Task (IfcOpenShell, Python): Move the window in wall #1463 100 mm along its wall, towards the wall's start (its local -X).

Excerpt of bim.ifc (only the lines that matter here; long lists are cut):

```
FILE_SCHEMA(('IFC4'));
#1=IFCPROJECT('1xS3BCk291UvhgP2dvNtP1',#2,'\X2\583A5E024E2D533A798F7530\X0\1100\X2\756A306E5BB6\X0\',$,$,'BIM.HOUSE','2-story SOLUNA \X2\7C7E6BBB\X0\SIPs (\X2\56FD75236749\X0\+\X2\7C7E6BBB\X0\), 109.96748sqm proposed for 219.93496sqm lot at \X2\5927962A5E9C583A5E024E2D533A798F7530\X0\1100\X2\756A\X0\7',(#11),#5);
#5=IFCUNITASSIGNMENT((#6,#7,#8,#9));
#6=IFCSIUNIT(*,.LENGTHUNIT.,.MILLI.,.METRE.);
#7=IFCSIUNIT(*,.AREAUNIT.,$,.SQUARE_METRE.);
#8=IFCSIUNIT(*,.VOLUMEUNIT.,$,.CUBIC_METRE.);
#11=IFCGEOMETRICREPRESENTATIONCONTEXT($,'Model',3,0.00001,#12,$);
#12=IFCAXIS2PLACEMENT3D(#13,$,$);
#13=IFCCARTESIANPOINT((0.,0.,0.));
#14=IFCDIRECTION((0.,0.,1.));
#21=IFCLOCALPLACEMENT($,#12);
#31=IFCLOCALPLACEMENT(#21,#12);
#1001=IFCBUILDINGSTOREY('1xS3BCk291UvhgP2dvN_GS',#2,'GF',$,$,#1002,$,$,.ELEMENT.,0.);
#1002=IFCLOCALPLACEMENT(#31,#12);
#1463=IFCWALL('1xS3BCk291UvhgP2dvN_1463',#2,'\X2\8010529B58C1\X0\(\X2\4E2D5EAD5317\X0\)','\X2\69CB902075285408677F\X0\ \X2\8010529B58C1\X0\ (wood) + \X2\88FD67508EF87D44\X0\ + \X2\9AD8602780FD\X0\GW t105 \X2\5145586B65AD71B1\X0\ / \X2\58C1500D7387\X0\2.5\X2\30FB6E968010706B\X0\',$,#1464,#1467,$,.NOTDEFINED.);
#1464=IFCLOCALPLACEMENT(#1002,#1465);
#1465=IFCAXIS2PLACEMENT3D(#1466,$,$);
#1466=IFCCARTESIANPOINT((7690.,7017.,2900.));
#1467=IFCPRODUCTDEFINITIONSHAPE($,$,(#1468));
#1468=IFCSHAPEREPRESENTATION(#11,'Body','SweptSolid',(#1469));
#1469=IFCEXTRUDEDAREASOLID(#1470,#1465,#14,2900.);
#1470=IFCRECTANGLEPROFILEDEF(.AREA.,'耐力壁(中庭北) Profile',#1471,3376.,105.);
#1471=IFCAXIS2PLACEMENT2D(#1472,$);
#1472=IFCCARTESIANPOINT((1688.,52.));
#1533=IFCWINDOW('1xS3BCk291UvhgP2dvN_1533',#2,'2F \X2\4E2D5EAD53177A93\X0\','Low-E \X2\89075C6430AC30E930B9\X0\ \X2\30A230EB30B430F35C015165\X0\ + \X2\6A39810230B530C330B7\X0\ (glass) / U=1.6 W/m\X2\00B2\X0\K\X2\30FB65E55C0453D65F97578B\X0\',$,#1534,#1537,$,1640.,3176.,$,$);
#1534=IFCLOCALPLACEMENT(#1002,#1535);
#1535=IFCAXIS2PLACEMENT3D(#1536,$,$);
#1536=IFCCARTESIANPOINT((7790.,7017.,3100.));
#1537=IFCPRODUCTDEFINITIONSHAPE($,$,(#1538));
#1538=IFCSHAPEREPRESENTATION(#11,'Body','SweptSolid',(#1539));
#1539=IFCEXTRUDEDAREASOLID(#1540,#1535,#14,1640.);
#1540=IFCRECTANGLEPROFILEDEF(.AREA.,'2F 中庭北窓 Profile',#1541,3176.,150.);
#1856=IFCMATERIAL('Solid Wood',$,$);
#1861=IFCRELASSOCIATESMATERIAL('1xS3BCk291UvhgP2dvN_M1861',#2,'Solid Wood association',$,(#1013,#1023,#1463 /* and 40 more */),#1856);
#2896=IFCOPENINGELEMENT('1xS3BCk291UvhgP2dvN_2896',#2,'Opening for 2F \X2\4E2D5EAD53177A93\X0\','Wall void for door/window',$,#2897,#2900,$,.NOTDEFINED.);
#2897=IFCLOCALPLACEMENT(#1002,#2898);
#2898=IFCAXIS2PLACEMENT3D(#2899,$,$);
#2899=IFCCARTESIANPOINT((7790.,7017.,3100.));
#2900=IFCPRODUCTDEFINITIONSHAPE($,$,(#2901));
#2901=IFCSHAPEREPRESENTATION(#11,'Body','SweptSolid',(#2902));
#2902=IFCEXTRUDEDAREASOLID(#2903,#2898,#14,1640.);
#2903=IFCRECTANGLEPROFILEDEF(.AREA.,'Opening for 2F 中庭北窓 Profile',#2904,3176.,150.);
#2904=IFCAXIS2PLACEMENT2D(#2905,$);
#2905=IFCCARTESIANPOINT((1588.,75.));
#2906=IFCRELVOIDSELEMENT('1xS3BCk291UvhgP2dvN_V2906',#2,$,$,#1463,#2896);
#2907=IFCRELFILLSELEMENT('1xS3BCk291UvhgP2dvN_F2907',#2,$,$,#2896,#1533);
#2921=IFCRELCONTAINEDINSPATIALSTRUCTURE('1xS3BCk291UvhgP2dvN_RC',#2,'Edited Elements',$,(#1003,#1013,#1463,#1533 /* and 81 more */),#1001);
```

```python
import ifcopenshell
import ifcopenshell.api.geometry
import ifcopenshell.util.placement
import ifcopenshell.util.unit

model = ifcopenshell.open("bim.ifc")
unit_scale = ifcopenshell.util.unit.calculate_unit_scale(model)

window = model.by_guid("1xS3BCk291UvhgP2dvN_1533")
opening = window.FillsVoids[0].RelatingOpeningElement
wall = opening.VoidsElements[0].RelatingBuildingElement

wall_matrix = ifcopenshell.util.placement.get_local_placement(wall.ObjectPlacement)
shift = wall_matrix[:3, 0] * -0.1 / unit_scale
before = ifcopenshell.util.placement.get_local_placement(window.ObjectPlacement)[:3, 3].copy()

# The window is not placed relative to its opening, so move both.
for product in (opening, window):
    matrix = ifcopenshell.util.placement.get_local_placement(product.ObjectPlacement)
    matrix[:3, 3] += shift
    ifcopenshell.api.geometry.edit_object_placement(model, product=product, matrix=matrix, is_si=False)

after = ifcopenshell.util.placement.get_local_placement(window.ObjectPlacement)[:3, 3]
print("window moved by", (after - before).round(3) + 0.0)

model.write("bim-out.ifc")
```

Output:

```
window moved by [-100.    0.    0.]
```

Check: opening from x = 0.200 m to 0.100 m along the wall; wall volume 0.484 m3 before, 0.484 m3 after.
